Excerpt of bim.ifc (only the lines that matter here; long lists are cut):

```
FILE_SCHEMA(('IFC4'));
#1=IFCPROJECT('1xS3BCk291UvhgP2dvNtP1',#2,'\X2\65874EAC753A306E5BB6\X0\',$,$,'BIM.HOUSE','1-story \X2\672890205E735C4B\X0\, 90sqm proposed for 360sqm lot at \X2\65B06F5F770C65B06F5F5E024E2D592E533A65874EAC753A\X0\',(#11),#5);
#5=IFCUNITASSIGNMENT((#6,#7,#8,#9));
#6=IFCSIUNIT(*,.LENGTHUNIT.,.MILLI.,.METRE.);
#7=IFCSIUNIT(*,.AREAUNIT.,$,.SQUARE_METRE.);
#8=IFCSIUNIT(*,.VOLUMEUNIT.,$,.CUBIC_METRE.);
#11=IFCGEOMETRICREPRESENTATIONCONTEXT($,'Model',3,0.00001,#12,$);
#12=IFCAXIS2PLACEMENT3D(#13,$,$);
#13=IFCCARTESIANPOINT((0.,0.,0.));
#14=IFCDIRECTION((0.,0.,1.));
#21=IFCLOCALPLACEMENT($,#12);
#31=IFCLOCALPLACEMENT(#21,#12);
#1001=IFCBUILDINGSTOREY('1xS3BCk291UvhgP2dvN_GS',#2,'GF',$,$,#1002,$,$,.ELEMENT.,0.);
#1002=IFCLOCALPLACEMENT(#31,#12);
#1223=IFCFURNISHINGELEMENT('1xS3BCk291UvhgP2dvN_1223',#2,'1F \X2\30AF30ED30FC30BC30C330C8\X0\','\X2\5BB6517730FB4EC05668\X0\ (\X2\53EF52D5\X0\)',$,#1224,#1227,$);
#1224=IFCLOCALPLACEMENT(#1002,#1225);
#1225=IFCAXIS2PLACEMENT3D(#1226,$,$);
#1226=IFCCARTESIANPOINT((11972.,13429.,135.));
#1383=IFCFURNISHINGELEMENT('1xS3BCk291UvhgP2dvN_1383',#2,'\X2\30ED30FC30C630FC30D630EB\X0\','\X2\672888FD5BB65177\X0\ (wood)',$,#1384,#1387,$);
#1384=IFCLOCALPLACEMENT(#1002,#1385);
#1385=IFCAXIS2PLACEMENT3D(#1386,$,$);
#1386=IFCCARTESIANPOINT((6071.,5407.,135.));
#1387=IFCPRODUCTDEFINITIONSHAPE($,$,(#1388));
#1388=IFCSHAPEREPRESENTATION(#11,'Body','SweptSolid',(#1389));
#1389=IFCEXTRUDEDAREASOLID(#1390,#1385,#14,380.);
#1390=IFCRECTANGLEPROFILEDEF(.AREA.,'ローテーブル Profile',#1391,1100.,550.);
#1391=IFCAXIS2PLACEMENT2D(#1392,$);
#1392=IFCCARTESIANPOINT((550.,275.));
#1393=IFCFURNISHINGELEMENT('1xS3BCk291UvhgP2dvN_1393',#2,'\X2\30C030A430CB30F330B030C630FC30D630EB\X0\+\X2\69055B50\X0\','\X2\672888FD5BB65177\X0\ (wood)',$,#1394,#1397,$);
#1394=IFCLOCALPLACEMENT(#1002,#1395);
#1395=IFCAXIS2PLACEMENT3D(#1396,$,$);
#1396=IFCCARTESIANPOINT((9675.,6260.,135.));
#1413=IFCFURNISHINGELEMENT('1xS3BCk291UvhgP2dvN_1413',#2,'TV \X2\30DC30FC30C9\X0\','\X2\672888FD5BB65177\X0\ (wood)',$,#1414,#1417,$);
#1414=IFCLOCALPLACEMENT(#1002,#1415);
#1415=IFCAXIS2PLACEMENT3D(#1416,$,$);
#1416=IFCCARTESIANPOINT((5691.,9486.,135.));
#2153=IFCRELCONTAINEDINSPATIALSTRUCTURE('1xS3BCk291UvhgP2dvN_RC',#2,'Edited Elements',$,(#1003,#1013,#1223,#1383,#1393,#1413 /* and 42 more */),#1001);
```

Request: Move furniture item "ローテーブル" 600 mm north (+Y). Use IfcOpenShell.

```python
import ifcopenshell
import ifcopenshell.api.geometry
import ifcopenshell.util.placement

model = ifcopenshell.open("bim.ifc")

item = model.by_guid("1xS3BCk291UvhgP2dvN_1383")
matrix = ifcopenshell.util.placement.get_local_placement(item.ObjectPlacement)
matrix[1, 3] += 600.0
ifcopenshell.api.geometry.edit_object_placement(model, product=item, matrix=matrix, is_si=False)

print(ifcopenshell.util.placement.get_local_placement(item.ObjectPlacement).round(3) + 0.0)

model.write("bim_v2.ifc")
```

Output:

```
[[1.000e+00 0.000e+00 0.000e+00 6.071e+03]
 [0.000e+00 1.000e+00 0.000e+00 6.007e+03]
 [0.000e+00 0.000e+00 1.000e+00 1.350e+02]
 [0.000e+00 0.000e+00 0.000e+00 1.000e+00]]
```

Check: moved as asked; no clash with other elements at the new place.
